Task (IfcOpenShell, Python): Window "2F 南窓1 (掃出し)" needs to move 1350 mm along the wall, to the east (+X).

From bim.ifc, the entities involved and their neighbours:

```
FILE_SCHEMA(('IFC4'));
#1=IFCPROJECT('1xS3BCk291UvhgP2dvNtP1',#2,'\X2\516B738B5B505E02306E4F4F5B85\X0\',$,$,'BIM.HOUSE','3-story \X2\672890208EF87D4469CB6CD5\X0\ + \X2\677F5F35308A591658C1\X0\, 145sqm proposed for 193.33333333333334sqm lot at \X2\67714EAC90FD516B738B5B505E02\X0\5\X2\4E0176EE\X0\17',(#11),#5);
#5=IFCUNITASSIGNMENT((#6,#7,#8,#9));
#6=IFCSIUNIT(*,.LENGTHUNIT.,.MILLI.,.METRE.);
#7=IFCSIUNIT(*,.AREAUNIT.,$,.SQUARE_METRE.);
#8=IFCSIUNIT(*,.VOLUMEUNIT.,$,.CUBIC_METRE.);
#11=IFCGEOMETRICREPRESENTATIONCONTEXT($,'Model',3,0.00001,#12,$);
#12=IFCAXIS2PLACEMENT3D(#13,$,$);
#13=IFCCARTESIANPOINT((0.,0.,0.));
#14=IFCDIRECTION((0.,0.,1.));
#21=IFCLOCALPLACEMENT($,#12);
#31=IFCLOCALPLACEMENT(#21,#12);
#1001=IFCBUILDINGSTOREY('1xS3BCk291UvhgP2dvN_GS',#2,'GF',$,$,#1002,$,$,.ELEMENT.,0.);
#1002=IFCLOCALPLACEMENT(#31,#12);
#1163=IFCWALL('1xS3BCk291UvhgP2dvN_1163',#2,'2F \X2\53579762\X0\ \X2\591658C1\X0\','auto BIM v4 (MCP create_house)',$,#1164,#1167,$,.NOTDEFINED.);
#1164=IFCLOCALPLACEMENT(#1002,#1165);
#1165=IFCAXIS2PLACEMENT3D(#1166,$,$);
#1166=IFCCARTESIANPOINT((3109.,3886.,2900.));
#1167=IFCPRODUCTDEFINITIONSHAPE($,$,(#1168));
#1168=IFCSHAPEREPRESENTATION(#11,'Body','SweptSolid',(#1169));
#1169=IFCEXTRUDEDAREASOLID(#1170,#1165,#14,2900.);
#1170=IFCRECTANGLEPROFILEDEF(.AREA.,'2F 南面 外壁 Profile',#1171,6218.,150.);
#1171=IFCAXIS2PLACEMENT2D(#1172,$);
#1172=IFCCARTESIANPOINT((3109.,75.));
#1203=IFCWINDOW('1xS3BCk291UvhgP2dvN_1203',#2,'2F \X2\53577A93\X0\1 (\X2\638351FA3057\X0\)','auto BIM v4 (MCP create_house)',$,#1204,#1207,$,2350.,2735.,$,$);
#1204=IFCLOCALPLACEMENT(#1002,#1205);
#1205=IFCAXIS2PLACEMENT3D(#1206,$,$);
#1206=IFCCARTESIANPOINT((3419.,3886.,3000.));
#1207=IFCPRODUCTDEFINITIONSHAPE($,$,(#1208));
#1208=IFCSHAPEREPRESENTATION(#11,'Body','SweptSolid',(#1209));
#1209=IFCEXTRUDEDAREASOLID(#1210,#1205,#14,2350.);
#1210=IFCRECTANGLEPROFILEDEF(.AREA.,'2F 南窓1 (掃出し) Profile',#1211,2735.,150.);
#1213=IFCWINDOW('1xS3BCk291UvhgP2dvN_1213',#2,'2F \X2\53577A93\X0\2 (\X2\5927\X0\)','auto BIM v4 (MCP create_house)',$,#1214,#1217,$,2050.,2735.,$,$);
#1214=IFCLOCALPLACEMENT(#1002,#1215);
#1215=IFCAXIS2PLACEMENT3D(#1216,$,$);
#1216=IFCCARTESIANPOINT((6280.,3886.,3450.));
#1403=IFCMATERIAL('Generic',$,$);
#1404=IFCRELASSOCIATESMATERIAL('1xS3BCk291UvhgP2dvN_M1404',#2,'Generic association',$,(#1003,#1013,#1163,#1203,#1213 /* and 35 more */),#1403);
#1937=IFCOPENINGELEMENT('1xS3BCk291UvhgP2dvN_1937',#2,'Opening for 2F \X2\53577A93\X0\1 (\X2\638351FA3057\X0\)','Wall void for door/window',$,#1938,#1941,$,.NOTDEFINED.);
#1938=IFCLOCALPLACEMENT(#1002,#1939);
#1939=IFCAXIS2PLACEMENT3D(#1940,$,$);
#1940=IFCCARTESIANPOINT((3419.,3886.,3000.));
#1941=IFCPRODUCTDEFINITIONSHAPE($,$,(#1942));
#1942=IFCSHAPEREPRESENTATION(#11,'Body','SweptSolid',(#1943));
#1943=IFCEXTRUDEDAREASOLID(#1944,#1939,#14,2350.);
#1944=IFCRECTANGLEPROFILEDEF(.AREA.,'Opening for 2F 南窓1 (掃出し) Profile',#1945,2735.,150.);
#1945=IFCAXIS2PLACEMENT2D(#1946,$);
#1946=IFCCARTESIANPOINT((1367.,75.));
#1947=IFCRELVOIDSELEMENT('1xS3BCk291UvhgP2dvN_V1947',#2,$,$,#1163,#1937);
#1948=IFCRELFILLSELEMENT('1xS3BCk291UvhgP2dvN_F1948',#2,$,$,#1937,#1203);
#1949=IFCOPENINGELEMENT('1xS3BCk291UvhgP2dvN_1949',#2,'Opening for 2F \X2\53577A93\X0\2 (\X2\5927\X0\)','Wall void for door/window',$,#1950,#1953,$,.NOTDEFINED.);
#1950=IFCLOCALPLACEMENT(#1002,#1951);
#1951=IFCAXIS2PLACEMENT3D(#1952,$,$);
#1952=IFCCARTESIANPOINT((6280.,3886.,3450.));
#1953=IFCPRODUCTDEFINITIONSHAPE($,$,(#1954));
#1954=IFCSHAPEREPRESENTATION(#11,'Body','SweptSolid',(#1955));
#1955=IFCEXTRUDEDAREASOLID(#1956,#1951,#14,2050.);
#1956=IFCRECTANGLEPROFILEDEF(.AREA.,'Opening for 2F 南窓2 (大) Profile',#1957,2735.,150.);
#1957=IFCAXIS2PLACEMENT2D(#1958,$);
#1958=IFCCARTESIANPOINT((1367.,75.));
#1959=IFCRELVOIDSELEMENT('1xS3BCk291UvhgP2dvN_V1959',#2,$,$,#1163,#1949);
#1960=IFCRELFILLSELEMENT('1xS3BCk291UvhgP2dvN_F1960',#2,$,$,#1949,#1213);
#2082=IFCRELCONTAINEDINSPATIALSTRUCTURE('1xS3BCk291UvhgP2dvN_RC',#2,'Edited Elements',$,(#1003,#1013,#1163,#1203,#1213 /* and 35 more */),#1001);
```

```python
import ifcopenshell
import ifcopenshell.api.geometry
import ifcopenshell.util.placement

model = ifcopenshell.open("bim.ifc")

window = model.by_guid("1xS3BCk291UvhgP2dvN_1203")
opening = window.FillsVoids[0].RelatingOpeningElement
wall = opening.VoidsElements[0].RelatingBuildingElement

wall_matrix = ifcopenshell.util.placement.get_local_placement(wall.ObjectPlacement)
shift = wall_matrix[:3, 0] * 1350.0
before = ifcopenshell.util.placement.get_local_placement(window.ObjectPlacement)[:3, 3].copy()

# The window is not placed relative to its opening, so move both.
for product in (opening, window):
    matrix = ifcopenshell.util.placement.get_local_placement(product.ObjectPlacement)
    matrix[:3, 3] += shift
    ifcopenshell.api.geometry.edit_object_placement(model, product=product, matrix=matrix, is_si=False)

after = ifcopenshell.util.placement.get_local_placement(window.ObjectPlacement)[:3, 3]
print("window moved by", (after - before).round(3) + 0.0)

model.write("bim_edited.ifc")
```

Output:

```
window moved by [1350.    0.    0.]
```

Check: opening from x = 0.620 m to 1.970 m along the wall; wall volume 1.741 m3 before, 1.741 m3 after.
